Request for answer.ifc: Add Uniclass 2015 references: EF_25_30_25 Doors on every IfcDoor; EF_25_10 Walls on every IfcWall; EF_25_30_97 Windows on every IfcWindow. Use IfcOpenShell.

First a look at what the model holds.

```python
import ifcopenshell

model = ifcopenshell.open("answer.ifc")
print(model.schema)
print("classifications:", [c.Name for c in model.by_type("IfcClassification")])
for ifc_class in ("IfcDoor", "IfcRoof", "IfcStair", "IfcWall", "IfcWindow"):
    print(ifc_class, len(model.by_type(ifc_class)))
```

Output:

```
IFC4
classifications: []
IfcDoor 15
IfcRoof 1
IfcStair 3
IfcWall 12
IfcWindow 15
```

```python
import ifcopenshell
import ifcopenshell.api.classification

model = ifcopenshell.open("answer.ifc")

system = ifcopenshell.api.classification.add_classification(model, classification="Uniclass 2015")

codes = {
    "IfcDoor": ("EF_25_30_25", "Doors"),
    "IfcWall": ("EF_25_10", "Walls"),
    "IfcWindow": ("EF_25_30_97", "Windows"),
}
for ifc_class, (code, name) in codes.items():
    products = model.by_type(ifc_class)
    ifcopenshell.api.classification.add_reference(
        model, products=products, classification=system, identification=code, name=name
    )
    print(code, len(products))

model.write("answer-out.ifc")
```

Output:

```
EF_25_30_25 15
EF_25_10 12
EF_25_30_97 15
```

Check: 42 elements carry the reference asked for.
